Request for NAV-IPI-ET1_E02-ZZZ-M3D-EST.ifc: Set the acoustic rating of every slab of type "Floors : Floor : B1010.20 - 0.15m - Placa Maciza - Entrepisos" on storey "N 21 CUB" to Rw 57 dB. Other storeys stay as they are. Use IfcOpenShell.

First a look at what the model holds.

```python
import ifcopenshell
import ifcopenshell.util.element

model = ifcopenshell.open("NAV-IPI-ET1_E02-ZZZ-M3D-EST.ifc")
print(model.schema)
storey = next(s for s in model.by_type("IfcBuildingStorey") if s.Name == "N 21 CUB")
slabs = [e for e in ifcopenshell.util.element.get_decomposition(storey) if e.is_a("IfcSlab")]
seen = {}
for e in slabs:
    element_type = ifcopenshell.util.element.get_type(e)
    key = (element_type.Name if element_type != e and element_type else None, ifcopenshell.util.element.get_pset(e, "Pset_SlabCommon", "AcousticRating"))
    seen[key] = seen.get(key, 0) + 1
for (name, value), count in sorted(seen.items(), key=str):
    print(count, "x", name, "|", value)
```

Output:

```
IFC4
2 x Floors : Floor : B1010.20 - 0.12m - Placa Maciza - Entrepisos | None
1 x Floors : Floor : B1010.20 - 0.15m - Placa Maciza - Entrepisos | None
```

```python
import ifcopenshell
import ifcopenshell.api.pset
import ifcopenshell.util.element

model = ifcopenshell.open("NAV-IPI-ET1_E02-ZZZ-M3D-EST.ifc")

storey = next(s for s in model.by_type("IfcBuildingStorey") if s.Name == "N 21 CUB")
slabs = [e for e in ifcopenshell.util.element.get_decomposition(storey) if e.is_a("IfcSlab")]

count = 0
for e in slabs:
    element_type = ifcopenshell.util.element.get_type(e)
    if element_type in (None, e) or element_type.Name != "Floors : Floor : B1010.20 - 0.15m - Placa Maciza - Entrepisos":
        continue
    # add_pset returns the element's existing set when there is one.
    pset = ifcopenshell.api.pset.add_pset(model, product=e, name="Pset_SlabCommon")
    ifcopenshell.api.pset.edit_pset(model, pset=pset, properties={"AcousticRating": "Rw 57 dB"})
    count += 1

print(count, "slabs updated")

model.write("NAV-IPI-ET1_E02-ZZZ-M3D-EST_rev.ifc")
```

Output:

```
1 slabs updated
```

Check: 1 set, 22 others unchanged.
